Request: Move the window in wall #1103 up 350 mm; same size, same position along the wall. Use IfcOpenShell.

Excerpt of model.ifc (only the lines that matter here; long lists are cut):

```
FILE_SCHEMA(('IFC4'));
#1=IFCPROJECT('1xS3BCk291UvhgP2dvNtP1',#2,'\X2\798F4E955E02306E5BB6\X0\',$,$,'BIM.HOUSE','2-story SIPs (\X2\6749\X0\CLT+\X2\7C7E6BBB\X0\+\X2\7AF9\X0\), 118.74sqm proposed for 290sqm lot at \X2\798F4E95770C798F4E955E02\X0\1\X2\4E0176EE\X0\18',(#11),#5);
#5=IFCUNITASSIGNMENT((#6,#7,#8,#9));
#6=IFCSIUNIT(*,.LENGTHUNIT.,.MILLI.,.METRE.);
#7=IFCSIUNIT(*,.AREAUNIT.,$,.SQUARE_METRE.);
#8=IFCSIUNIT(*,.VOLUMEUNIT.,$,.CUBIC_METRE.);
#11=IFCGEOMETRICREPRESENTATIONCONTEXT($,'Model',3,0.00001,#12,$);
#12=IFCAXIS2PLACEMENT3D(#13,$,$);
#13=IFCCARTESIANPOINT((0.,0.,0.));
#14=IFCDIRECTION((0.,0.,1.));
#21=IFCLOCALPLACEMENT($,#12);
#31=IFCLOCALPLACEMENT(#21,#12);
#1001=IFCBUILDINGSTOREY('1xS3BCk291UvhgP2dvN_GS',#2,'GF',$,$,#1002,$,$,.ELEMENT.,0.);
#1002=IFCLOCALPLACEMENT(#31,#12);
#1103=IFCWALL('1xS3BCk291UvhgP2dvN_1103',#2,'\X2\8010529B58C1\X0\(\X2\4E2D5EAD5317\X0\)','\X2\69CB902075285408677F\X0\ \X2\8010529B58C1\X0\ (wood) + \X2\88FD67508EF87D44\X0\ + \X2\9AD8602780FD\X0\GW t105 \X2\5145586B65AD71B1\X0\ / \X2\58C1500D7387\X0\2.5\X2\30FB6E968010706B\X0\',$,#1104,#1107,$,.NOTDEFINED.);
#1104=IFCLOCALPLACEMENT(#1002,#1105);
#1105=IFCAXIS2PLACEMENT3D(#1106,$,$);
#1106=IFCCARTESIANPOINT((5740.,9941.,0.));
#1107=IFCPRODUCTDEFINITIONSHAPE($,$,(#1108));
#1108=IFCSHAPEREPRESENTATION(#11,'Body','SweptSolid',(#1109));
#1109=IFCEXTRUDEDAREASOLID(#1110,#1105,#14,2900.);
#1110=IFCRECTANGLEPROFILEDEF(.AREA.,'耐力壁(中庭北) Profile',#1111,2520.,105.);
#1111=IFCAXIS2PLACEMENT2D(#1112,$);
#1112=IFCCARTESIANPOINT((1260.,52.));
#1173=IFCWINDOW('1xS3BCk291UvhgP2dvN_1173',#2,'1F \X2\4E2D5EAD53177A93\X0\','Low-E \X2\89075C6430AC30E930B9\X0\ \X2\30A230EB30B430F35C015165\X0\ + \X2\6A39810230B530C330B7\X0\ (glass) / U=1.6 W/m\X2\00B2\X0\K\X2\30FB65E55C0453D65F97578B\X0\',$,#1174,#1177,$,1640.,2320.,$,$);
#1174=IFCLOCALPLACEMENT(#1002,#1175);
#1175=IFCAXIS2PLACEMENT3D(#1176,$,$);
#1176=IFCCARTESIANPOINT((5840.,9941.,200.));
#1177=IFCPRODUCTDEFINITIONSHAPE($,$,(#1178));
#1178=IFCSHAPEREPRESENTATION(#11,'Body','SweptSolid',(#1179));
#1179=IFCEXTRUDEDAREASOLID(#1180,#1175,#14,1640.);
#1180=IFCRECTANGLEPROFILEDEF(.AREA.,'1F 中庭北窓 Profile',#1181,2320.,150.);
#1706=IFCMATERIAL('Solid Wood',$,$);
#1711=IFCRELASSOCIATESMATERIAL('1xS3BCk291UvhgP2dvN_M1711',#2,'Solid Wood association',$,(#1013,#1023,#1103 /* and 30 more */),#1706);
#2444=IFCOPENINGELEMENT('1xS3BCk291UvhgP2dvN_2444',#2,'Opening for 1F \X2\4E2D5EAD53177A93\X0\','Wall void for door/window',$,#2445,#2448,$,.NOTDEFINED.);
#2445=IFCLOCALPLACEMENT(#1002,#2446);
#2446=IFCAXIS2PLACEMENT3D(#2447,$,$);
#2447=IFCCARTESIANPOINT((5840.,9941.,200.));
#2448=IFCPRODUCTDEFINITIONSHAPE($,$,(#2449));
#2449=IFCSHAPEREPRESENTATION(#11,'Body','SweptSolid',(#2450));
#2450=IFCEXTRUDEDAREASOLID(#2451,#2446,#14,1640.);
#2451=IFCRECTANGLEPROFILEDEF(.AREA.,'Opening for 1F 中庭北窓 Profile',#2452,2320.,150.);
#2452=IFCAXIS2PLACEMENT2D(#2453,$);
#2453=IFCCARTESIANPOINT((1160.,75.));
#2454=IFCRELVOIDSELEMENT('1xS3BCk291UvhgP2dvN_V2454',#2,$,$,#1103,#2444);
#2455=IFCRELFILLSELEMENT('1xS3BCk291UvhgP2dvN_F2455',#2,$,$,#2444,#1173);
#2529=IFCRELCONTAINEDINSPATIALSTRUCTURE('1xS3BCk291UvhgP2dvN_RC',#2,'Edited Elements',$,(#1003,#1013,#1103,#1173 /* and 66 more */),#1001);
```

```python
import numpy as np
import ifcopenshell
import ifcopenshell.api.geometry
import ifcopenshell.util.placement
import ifcopenshell.util.unit

model = ifcopenshell.open("model.ifc")
unit_scale = ifcopenshell.util.unit.calculate_unit_scale(model)

window = model.by_id(1173)
opening = window.FillsVoids[0].RelatingOpeningElement
dz = 350.0

shift = np.array([0.0, 0.0, dz])
# The window is not placed relative to its opening, so move both.
for product in (opening, window):
    matrix = ifcopenshell.util.placement.get_local_placement(product.ObjectPlacement)
    matrix[:3, 3] += shift
    ifcopenshell.api.geometry.edit_object_placement(model, product=product, matrix=matrix, is_si=False)

print(f"moved by {dz * unit_scale:+.3f} m")

model.write("model_edited.ifc")
```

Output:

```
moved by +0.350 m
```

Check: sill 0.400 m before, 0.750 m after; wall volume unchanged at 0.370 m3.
